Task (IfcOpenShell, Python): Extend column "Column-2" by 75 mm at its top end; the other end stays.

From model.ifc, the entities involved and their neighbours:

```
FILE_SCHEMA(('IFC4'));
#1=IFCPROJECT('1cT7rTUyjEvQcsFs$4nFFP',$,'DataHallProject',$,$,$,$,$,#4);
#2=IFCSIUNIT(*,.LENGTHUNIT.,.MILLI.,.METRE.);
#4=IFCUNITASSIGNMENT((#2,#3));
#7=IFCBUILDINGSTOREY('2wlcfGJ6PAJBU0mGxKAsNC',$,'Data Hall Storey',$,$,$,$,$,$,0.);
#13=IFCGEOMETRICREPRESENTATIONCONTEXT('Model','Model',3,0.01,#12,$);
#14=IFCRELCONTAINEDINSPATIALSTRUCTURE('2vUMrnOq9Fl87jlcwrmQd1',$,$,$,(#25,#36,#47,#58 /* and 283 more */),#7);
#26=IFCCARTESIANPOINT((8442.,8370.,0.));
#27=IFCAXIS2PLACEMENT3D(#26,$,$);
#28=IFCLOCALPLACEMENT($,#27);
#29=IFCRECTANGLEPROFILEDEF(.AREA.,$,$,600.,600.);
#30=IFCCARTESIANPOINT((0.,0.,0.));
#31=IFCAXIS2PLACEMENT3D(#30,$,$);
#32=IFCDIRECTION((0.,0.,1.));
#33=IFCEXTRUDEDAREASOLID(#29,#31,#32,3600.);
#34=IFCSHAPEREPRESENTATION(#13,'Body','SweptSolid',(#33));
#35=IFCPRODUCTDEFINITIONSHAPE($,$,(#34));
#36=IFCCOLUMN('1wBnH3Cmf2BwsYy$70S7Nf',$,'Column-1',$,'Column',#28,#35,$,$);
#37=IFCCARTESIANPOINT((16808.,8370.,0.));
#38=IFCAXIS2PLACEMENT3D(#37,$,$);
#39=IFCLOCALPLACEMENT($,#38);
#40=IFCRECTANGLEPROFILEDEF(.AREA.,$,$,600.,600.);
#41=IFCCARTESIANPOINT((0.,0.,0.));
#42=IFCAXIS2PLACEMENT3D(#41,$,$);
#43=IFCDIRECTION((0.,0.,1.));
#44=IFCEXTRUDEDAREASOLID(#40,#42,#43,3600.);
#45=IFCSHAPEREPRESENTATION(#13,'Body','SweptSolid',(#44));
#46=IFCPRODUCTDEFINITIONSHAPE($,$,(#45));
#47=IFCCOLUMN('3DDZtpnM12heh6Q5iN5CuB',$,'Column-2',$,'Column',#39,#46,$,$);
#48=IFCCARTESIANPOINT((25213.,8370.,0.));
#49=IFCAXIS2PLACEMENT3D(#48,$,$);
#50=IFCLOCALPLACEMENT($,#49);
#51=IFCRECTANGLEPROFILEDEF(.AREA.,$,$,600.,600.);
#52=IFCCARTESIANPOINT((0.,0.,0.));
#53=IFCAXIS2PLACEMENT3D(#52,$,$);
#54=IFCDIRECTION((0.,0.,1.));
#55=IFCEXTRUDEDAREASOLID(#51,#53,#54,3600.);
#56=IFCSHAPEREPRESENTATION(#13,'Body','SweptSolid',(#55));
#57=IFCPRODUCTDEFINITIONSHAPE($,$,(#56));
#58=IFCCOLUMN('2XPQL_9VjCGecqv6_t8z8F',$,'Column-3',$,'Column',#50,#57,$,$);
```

```python
import ifcopenshell
import ifcopenshell.util.unit

model = ifcopenshell.open("model.ifc")
unit_scale = ifcopenshell.util.unit.calculate_unit_scale(model)

member = model.by_guid("3DDZtpnM12heh6Q5iN5CuB")
change = 0.075 / unit_scale

# The extrusion runs towards the end named, so only its depth changes.
body = next(r for r in member.Representation.Representations if r.RepresentationIdentifier == "Body")
solid = body.Items[0]
old_length = solid.Depth
solid.Depth += change

print(f"length {old_length:g} -> {solid.Depth:g}")

model.write("model_rev.ifc")
```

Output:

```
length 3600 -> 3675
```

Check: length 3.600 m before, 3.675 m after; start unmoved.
